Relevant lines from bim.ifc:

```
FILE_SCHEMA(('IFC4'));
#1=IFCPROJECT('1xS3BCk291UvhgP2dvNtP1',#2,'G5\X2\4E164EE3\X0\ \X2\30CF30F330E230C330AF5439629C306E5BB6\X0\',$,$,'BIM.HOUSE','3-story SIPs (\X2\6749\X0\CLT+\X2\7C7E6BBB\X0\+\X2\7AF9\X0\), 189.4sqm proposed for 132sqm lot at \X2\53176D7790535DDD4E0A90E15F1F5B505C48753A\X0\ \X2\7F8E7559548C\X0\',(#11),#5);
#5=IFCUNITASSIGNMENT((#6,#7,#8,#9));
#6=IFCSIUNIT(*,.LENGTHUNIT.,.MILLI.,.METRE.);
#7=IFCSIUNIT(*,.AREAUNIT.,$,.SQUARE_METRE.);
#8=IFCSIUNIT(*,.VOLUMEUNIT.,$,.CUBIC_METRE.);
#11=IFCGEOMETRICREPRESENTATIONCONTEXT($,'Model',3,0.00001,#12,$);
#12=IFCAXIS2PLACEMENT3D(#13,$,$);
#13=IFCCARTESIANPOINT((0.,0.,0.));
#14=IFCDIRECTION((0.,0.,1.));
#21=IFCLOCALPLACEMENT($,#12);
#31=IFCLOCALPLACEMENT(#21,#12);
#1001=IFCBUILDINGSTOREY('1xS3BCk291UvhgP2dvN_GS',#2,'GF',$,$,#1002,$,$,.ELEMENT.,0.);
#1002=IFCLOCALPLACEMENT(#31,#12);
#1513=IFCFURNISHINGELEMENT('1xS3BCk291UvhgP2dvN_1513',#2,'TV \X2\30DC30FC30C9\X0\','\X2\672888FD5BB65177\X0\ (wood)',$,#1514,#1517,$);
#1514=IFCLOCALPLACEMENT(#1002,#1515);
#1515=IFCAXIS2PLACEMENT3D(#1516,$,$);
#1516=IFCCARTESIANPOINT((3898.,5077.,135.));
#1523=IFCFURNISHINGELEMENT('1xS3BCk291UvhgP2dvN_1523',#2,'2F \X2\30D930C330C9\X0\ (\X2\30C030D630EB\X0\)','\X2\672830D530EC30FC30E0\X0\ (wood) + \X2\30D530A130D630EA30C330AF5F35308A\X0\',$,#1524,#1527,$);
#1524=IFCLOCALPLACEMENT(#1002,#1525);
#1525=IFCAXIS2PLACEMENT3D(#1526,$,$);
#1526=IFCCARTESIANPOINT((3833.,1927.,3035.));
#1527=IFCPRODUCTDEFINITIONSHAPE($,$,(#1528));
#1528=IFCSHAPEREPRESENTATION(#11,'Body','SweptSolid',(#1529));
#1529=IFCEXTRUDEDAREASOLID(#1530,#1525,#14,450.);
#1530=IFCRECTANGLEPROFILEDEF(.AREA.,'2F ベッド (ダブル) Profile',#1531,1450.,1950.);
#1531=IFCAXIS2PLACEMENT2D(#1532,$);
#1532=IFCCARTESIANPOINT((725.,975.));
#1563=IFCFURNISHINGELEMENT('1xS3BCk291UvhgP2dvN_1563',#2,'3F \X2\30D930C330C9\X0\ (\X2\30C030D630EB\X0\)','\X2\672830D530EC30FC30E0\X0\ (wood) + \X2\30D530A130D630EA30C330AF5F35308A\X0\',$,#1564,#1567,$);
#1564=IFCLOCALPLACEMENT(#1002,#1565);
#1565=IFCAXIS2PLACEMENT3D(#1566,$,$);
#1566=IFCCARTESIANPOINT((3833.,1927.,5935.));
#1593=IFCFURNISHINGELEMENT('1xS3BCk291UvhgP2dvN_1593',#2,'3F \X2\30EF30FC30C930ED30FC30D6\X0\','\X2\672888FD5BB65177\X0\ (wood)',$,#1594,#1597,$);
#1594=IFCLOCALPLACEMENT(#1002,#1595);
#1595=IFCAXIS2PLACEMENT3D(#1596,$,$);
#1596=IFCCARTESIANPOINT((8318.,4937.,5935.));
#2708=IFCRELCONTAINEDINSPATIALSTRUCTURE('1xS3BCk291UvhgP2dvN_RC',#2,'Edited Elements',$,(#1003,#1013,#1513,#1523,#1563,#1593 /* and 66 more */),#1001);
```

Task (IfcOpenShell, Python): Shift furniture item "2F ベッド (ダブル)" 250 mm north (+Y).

```python
import ifcopenshell
import ifcopenshell.api.geometry
import ifcopenshell.util.placement

model = ifcopenshell.open("bim.ifc")

item = model.by_guid("1xS3BCk291UvhgP2dvN_1523")
matrix = ifcopenshell.util.placement.get_local_placement(item.ObjectPlacement)
matrix[1, 3] += 250.0
ifcopenshell.api.geometry.edit_object_placement(model, product=item, matrix=matrix, is_si=False)

print(ifcopenshell.util.placement.get_local_placement(item.ObjectPlacement).round(3) + 0.0)

model.write("bim-out.ifc")
```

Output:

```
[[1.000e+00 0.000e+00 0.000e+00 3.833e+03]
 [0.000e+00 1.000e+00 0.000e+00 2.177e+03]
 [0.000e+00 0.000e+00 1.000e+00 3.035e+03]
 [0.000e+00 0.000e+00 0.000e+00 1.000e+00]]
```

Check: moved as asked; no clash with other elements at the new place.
